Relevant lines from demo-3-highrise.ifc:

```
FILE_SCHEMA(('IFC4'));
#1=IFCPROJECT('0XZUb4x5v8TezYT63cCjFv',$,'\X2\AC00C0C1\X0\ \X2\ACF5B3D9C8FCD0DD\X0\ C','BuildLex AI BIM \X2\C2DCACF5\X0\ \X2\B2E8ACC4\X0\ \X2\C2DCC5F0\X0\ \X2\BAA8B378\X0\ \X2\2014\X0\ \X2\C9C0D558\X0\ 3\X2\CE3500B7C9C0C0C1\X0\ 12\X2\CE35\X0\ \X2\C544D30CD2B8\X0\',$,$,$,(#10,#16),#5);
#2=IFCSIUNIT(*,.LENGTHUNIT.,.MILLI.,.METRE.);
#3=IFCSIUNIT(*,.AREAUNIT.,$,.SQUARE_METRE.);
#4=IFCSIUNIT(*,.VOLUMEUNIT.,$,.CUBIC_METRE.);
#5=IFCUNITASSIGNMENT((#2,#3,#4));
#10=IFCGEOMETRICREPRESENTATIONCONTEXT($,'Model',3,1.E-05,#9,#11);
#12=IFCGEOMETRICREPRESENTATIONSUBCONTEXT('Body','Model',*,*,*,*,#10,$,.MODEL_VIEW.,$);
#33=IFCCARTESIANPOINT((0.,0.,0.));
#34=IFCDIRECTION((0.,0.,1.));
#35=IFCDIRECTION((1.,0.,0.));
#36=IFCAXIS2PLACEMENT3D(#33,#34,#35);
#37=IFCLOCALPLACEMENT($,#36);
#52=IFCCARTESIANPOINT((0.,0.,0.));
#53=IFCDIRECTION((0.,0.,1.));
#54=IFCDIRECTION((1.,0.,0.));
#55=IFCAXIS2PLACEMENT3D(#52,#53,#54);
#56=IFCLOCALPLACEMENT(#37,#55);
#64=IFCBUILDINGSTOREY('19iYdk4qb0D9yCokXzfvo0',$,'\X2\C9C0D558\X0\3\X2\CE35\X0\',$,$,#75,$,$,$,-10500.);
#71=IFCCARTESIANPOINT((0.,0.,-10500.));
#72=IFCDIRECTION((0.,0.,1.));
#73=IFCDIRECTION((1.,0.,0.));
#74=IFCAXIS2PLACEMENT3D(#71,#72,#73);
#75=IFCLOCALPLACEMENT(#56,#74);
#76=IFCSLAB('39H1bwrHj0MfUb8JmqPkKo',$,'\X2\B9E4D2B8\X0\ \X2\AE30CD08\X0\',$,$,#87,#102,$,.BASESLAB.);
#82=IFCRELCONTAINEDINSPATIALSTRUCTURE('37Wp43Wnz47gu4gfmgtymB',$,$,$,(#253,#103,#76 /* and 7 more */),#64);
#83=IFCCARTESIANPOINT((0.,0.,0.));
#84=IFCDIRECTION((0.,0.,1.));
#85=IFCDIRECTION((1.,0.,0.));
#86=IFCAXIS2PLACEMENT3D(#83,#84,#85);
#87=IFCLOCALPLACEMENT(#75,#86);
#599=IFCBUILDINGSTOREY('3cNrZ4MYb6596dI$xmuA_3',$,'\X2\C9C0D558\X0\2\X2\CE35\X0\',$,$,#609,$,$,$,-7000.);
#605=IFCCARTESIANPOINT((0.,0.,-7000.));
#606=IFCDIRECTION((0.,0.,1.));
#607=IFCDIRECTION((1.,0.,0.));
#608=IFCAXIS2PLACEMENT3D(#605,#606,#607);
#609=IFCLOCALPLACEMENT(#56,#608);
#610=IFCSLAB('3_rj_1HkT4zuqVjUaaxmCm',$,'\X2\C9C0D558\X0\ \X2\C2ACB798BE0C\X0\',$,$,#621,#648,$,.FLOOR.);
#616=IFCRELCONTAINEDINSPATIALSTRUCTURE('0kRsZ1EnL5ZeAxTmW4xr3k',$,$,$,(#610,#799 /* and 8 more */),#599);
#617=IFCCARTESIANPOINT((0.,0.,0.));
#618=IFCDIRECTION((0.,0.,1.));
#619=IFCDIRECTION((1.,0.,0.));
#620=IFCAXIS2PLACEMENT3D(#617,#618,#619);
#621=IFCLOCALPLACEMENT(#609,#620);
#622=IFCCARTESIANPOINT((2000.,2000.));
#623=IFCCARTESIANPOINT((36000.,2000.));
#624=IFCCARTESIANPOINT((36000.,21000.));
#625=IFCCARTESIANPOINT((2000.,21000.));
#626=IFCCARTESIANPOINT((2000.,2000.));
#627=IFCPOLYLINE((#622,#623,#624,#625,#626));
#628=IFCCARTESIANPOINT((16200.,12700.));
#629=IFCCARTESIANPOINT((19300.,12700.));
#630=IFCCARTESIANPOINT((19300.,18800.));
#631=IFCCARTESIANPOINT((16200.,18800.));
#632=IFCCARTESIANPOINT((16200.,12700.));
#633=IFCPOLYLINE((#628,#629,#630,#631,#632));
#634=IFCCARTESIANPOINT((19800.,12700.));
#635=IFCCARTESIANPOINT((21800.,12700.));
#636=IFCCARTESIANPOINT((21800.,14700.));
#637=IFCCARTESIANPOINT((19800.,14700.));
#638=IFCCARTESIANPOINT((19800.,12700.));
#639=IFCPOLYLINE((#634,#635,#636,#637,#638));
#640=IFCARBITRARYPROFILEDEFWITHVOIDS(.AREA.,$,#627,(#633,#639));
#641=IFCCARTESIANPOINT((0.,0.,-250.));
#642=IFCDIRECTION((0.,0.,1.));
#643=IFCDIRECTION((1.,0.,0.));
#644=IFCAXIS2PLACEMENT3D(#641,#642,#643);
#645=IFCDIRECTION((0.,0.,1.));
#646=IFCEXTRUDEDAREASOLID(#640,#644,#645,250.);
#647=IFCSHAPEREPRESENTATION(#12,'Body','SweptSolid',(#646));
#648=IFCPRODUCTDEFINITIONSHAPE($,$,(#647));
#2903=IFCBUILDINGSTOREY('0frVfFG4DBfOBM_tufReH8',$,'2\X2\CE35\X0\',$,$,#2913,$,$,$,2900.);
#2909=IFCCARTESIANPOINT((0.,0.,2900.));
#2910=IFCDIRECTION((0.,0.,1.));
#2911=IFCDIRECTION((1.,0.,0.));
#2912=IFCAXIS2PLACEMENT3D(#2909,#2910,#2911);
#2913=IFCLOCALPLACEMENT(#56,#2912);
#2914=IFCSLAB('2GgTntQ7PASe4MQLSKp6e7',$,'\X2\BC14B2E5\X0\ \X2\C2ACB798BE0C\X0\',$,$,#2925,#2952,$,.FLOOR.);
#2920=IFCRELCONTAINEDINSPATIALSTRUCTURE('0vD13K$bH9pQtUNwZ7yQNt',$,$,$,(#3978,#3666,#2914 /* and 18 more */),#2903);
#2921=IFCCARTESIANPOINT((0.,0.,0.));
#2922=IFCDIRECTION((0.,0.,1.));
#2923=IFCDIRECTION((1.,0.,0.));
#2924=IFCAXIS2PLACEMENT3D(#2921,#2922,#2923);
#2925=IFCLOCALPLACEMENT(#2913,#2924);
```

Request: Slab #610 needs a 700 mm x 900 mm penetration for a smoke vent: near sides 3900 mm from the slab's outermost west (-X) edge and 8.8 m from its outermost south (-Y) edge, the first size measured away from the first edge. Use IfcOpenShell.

```python
import numpy as np
import ifcopenshell
import ifcopenshell.api.feature
import ifcopenshell.api.geometry
import ifcopenshell.api.root
import ifcopenshell.geom
import ifcopenshell.util.placement
import ifcopenshell.util.representation
import ifcopenshell.util.shape
import ifcopenshell.util.unit

model = ifcopenshell.open("demo-3-highrise.ifc")
unit_scale = ifcopenshell.util.unit.calculate_unit_scale(model)
settings = ifcopenshell.geom.settings()


def volume(element):
    """Net volume in cubic metres, openings subtracted."""
    shape = ifcopenshell.geom.create_shape(settings, element)
    return ifcopenshell.util.shape.get_volume(shape.geometry)


slab = model.by_guid("3_rj_1HkT4zuqVjUaaxmCm")
before = volume(slab)

# Extent in the slab's own axes, in metres. The edges named are its -X and -Y sides.
slab_shape = ifcopenshell.geom.create_shape(settings, slab)
vertices = ifcopenshell.util.shape.get_vertices(slab_shape.geometry)
x_min, y_min, bottom = vertices.min(axis=0)
top = vertices[:, 2].max()

opening = ifcopenshell.api.root.create_entity(model, ifc_class="IfcOpeningElement", name="Smoke vent opening", predefined_type="OPENING")
context = ifcopenshell.util.representation.get_context(model, "Model", "Body", "MODEL_VIEW")
width, depth = 0.7, 0.9
outline = [(0.0, 0.0), (width, 0.0), (width, depth), (0.0, depth), (0.0, 0.0)]
# Overshoot both faces by 50 mm so the cut is clean.
shape = ifcopenshell.api.geometry.add_slab_representation(
    model, context=context, depth=top - bottom + 0.1, polyline=outline
)
ifcopenshell.api.geometry.assign_representation(model, product=opening, representation=shape)

matrix = ifcopenshell.util.placement.get_local_placement(slab.ObjectPlacement)
matrix[:, 3] = matrix @ np.append(np.array([x_min + 3.9, y_min + 8.8, bottom - 0.05]) / unit_scale, 1.0)
ifcopenshell.api.geometry.edit_object_placement(model, product=opening, matrix=matrix, is_si=False)
ifcopenshell.api.feature.add_feature(model, feature=opening, element=slab)

after = volume(slab)

print(f"slab volume {before:.3f} -> {after:.3f} m3")

model.write("demo-3-highrise_rev.ifc")
```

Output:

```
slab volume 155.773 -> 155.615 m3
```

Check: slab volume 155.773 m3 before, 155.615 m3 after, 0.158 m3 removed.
